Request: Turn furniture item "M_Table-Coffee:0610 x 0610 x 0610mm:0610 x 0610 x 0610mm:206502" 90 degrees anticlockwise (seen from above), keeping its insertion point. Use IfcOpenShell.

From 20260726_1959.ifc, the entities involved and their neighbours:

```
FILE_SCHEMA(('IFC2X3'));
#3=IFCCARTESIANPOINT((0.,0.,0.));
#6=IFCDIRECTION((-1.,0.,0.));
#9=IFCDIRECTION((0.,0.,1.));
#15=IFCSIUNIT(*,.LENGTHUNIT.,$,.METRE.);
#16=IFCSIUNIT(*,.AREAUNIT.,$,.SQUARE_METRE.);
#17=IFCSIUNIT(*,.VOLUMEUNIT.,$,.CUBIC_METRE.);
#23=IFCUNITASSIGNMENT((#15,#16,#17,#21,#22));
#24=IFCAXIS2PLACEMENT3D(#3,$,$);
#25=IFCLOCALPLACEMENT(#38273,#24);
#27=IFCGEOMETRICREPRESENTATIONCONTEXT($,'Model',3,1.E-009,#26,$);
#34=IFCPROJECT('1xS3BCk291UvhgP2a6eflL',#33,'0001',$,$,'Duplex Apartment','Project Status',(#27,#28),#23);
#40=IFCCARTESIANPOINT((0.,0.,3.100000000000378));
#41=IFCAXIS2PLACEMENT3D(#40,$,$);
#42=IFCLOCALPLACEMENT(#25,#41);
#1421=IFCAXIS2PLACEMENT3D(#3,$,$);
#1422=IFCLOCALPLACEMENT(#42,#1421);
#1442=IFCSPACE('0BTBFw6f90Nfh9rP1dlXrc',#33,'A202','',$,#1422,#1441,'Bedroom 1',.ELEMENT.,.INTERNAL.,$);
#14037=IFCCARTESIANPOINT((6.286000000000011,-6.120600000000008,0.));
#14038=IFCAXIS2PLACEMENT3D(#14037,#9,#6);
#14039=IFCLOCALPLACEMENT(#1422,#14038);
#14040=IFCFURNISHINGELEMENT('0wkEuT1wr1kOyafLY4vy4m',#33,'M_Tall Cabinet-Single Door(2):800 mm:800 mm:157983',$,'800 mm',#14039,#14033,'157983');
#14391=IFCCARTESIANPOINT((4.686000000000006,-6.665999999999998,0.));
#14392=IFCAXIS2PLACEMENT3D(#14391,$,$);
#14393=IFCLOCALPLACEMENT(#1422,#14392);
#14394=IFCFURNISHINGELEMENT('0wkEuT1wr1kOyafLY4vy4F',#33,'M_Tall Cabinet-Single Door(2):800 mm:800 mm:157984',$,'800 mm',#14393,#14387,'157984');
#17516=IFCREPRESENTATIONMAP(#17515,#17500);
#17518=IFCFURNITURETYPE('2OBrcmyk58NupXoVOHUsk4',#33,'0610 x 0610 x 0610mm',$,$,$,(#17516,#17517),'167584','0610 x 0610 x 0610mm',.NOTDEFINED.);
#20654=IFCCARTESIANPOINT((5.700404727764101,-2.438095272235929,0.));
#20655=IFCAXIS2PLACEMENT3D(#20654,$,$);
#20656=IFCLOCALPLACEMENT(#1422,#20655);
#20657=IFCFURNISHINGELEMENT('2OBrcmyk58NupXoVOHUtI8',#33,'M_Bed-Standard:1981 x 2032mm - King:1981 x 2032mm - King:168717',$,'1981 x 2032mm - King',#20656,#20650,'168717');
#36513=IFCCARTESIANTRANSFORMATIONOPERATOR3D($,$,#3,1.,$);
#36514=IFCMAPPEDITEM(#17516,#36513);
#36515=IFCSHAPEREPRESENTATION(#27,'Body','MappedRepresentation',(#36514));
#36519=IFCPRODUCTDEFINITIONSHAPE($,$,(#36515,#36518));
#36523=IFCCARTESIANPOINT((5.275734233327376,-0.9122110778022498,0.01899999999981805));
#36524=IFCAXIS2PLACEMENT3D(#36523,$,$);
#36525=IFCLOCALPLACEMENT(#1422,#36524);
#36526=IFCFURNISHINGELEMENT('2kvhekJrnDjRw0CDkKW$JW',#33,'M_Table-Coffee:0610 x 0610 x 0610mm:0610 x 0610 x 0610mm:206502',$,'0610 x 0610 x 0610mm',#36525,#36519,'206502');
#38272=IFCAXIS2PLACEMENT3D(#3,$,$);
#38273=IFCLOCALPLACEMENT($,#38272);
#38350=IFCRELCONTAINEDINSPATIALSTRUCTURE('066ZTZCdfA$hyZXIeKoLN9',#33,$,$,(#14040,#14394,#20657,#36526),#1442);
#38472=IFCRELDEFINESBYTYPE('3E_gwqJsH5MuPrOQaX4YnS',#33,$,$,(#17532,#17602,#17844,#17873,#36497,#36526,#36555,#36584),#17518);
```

```python
import ifcopenshell
import ifcopenshell.api.geometry
import ifcopenshell.util.placement

model = ifcopenshell.open("20260726_1959.ifc")

item = model.by_guid("2kvhekJrnDjRw0CDkKW$JW")
matrix = ifcopenshell.util.placement.get_local_placement(item.ObjectPlacement)
matrix = matrix @ ifcopenshell.util.placement.rotation(90, "Z")
ifcopenshell.api.geometry.edit_object_placement(model, product=item, matrix=matrix, is_si=False)

print(ifcopenshell.util.placement.get_local_placement(item.ObjectPlacement).round(3) + 0.0)

model.write("20260726_1959_edited.ifc")
```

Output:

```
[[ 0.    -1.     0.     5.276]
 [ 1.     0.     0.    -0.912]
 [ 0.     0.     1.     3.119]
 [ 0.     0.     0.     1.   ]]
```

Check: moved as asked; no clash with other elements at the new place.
